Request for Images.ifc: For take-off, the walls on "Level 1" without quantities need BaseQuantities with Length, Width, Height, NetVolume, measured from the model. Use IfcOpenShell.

First a look at what the model holds.

```python
import ifcopenshell
import ifcopenshell.util.element
import ifcopenshell.util.unit

model = ifcopenshell.open("Images.ifc")
print(model.schema)
for unit_type in ("LENGTHUNIT", "AREAUNIT", "VOLUMEUNIT"):
    print(unit_type, ifcopenshell.util.unit.calculate_unit_scale(model, unit_type))
storey = next(s for s in model.by_type("IfcBuildingStorey") if s.Name == "Level 1")
walls = [e for e in ifcopenshell.util.element.get_decomposition(storey) if e.is_a("IfcWall")]
for e in sorted(walls, key=lambda e: e.id()):
    print(e.id(), e.is_a(), e.Name, list(ifcopenshell.util.element.get_psets(e, qtos_only=True)), sep=" | ")
```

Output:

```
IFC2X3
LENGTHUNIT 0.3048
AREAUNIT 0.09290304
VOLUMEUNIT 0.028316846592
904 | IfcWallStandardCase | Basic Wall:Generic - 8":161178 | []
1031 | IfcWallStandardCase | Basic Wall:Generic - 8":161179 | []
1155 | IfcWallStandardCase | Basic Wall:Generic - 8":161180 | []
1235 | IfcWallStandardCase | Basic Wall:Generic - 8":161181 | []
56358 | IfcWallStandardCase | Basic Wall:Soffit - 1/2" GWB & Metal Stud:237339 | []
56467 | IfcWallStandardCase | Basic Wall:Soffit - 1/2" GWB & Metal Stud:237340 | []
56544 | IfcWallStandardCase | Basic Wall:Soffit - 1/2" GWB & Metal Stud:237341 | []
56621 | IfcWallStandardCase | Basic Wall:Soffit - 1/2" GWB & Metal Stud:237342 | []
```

```python
import ifcopenshell
import ifcopenshell.api.pset
import ifcopenshell.geom
import ifcopenshell.util.element
import ifcopenshell.util.shape
import ifcopenshell.util.unit

model = ifcopenshell.open("Images.ifc")
unit_scale = ifcopenshell.util.unit.calculate_unit_scale(model)
volume_scale = ifcopenshell.util.unit.calculate_unit_scale(model, "VOLUMEUNIT")
settings = ifcopenshell.geom.settings()

storey = next(s for s in model.by_type("IfcBuildingStorey") if s.Name == "Level 1")
walls = [e for e in ifcopenshell.util.element.get_decomposition(storey) if e.is_a("IfcWall")]

for e in sorted(walls, key=lambda e: e.id()):
    if ifcopenshell.util.element.get_psets(e, qtos_only=True, should_inherit=False):
        continue
    # Geometry comes back in metres, in the element's own axes.
    shape = ifcopenshell.geom.create_shape(settings, e)
    values = {
        "Length": ifcopenshell.util.shape.get_x(shape.geometry) / unit_scale,
        "Width": ifcopenshell.util.shape.get_y(shape.geometry) / unit_scale,
        "Height": ifcopenshell.util.shape.get_z(shape.geometry) / unit_scale,
        "NetVolume": ifcopenshell.util.shape.get_volume(shape.geometry) / volume_scale,
    }
    qto = ifcopenshell.api.pset.add_qto(model, product=e, name="BaseQuantities")
    ifcopenshell.api.pset.edit_qto(model, qto=qto, properties=values)
    print(e.id(), {k: round(v, 3) for k, v in values.items()})

model.write("Images_edited.ifc")
```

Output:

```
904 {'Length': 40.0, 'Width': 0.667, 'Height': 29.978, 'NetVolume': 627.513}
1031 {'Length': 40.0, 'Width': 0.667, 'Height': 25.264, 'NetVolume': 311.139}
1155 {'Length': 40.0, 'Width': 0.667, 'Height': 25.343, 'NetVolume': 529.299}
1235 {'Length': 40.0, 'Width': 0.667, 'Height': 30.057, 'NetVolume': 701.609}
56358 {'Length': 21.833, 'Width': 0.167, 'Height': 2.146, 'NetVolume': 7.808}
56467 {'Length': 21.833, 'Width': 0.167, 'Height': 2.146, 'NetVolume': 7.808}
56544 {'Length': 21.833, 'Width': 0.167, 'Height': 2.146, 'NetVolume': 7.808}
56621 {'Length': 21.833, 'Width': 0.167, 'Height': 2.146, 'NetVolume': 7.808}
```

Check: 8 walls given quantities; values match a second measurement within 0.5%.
